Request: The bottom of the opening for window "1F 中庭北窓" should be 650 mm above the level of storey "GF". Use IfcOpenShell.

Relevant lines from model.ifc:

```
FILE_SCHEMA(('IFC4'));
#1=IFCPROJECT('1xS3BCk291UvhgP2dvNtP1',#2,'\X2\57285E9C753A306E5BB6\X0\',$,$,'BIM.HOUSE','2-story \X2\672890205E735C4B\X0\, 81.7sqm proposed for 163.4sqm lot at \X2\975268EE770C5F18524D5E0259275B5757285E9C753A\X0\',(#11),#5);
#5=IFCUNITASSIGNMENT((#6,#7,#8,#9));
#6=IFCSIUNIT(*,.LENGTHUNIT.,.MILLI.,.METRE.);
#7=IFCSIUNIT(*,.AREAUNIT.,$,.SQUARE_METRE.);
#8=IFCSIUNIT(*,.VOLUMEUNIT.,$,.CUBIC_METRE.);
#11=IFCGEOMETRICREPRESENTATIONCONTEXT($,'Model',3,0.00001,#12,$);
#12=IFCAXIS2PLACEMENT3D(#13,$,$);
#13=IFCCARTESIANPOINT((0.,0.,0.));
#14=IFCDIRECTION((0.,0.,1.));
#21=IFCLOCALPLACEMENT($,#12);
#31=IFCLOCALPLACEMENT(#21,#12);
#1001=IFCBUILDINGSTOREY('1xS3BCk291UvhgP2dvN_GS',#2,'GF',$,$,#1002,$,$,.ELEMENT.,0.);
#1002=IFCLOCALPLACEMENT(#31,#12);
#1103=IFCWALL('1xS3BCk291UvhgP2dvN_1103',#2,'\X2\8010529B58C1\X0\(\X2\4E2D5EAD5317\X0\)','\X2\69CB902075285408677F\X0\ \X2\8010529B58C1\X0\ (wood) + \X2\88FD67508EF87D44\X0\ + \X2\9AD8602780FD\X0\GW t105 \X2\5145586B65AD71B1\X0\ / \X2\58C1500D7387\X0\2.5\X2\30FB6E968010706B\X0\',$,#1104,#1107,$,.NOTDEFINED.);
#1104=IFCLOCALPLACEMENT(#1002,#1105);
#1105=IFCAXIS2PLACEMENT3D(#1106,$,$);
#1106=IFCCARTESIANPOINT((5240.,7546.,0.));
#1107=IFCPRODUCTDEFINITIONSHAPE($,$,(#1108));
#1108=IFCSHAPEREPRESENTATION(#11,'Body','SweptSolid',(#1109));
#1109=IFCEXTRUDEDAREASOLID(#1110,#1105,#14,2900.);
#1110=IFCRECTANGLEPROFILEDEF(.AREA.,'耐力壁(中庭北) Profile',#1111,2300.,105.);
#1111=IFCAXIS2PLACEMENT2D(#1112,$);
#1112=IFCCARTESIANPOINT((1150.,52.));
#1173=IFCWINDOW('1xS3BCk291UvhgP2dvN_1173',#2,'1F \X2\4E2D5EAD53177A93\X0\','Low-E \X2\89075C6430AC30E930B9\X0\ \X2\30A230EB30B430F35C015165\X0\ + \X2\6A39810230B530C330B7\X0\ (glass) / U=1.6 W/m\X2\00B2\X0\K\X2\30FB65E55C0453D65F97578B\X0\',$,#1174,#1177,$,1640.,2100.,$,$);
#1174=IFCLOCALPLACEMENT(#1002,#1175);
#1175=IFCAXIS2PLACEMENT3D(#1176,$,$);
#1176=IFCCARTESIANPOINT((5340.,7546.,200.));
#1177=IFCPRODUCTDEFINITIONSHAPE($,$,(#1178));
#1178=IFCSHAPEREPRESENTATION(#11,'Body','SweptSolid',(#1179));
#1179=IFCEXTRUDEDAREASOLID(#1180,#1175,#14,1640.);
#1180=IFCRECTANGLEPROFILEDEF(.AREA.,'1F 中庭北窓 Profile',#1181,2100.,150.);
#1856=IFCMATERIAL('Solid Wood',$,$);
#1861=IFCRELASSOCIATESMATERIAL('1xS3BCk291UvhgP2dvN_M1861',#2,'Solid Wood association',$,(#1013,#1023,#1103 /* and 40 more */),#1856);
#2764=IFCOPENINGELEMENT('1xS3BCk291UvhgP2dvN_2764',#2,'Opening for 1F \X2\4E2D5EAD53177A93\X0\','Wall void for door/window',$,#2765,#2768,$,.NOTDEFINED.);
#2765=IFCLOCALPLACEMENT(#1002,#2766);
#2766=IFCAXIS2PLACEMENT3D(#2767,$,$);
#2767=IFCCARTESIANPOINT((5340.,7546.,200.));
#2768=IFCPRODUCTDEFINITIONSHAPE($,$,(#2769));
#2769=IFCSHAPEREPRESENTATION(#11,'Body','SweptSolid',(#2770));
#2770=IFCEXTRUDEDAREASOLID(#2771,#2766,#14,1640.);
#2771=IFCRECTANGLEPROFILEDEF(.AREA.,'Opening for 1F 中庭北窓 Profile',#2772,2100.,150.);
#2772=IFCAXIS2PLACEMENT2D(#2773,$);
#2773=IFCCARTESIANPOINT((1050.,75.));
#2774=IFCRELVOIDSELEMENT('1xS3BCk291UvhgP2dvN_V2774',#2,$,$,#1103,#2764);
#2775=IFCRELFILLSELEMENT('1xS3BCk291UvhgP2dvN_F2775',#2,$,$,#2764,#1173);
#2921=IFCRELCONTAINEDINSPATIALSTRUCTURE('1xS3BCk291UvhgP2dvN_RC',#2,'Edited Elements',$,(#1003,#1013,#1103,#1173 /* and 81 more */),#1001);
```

```python
import numpy as np
import ifcopenshell
import ifcopenshell.api.geometry
import ifcopenshell.geom
import ifcopenshell.util.element
import ifcopenshell.util.placement
import ifcopenshell.util.shape
import ifcopenshell.util.unit

model = ifcopenshell.open("model.ifc")
unit_scale = ifcopenshell.util.unit.calculate_unit_scale(model)

window = model.by_id(1173)
opening = window.FillsVoids[0].RelatingOpeningElement
storey = ifcopenshell.util.element.get_container(window, ifc_class="IfcBuildingStorey")
level = ifcopenshell.util.placement.get_local_placement(storey.ObjectPlacement)[2, 3]

# The opening's origin need not be at the sill, so measure its lowest point.
shape = ifcopenshell.geom.create_shape(ifcopenshell.geom.settings(), opening)
bottom = ifcopenshell.util.shape.get_shape_bottom_elevation(shape, shape.geometry) / unit_scale
dz = level + 650.0 - bottom

shift = np.array([0.0, 0.0, dz])
# The window is not placed relative to its opening, so move both.
for product in (opening, window):
    matrix = ifcopenshell.util.placement.get_local_placement(product.ObjectPlacement)
    matrix[:3, 3] += shift
    ifcopenshell.api.geometry.edit_object_placement(model, product=product, matrix=matrix, is_si=False)

print(f"moved by {dz * unit_scale:+.3f} m")

model.write("model_updated.ifc")
```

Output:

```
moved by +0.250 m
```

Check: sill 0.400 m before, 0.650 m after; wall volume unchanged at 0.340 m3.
